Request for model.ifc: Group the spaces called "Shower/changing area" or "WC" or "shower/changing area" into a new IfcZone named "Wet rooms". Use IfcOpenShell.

First a look at what the model holds.

```python
import ifcopenshell

model = ifcopenshell.open("model.ifc")
print(model.schema)
seen = {}
for space in model.by_type("IfcSpace"):
    seen[space.LongName] = seen.get(space.LongName, 0) + 1
for name, count in sorted(seen.items(), key=str):
    print(count, "x", name)
print("zones:", [z.Name for z in model.by_type("IfcZone")][:20])
```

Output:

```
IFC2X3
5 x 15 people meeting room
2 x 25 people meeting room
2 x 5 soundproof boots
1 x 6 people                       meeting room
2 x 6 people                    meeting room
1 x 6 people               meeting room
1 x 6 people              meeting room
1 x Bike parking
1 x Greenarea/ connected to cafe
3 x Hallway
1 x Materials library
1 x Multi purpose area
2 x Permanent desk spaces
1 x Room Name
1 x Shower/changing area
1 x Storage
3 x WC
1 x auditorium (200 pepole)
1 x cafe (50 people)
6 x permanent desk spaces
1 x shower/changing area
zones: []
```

```python
import ifcopenshell
import ifcopenshell.api.group
import ifcopenshell.api.root

model = ifcopenshell.open("model.ifc")

names = {"Shower/changing area", "WC", "shower/changing area"}
spaces = [s for s in model.by_type("IfcSpace") if s.LongName in names]

zone = ifcopenshell.api.root.create_entity(model, ifc_class="IfcZone", name="Wet rooms")
ifcopenshell.api.group.assign_group(model, products=spaces, group=zone)
print(len(spaces), "spaces in", zone.Name)

model.write("model_v2.ifc")
```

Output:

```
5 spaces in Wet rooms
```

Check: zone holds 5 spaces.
